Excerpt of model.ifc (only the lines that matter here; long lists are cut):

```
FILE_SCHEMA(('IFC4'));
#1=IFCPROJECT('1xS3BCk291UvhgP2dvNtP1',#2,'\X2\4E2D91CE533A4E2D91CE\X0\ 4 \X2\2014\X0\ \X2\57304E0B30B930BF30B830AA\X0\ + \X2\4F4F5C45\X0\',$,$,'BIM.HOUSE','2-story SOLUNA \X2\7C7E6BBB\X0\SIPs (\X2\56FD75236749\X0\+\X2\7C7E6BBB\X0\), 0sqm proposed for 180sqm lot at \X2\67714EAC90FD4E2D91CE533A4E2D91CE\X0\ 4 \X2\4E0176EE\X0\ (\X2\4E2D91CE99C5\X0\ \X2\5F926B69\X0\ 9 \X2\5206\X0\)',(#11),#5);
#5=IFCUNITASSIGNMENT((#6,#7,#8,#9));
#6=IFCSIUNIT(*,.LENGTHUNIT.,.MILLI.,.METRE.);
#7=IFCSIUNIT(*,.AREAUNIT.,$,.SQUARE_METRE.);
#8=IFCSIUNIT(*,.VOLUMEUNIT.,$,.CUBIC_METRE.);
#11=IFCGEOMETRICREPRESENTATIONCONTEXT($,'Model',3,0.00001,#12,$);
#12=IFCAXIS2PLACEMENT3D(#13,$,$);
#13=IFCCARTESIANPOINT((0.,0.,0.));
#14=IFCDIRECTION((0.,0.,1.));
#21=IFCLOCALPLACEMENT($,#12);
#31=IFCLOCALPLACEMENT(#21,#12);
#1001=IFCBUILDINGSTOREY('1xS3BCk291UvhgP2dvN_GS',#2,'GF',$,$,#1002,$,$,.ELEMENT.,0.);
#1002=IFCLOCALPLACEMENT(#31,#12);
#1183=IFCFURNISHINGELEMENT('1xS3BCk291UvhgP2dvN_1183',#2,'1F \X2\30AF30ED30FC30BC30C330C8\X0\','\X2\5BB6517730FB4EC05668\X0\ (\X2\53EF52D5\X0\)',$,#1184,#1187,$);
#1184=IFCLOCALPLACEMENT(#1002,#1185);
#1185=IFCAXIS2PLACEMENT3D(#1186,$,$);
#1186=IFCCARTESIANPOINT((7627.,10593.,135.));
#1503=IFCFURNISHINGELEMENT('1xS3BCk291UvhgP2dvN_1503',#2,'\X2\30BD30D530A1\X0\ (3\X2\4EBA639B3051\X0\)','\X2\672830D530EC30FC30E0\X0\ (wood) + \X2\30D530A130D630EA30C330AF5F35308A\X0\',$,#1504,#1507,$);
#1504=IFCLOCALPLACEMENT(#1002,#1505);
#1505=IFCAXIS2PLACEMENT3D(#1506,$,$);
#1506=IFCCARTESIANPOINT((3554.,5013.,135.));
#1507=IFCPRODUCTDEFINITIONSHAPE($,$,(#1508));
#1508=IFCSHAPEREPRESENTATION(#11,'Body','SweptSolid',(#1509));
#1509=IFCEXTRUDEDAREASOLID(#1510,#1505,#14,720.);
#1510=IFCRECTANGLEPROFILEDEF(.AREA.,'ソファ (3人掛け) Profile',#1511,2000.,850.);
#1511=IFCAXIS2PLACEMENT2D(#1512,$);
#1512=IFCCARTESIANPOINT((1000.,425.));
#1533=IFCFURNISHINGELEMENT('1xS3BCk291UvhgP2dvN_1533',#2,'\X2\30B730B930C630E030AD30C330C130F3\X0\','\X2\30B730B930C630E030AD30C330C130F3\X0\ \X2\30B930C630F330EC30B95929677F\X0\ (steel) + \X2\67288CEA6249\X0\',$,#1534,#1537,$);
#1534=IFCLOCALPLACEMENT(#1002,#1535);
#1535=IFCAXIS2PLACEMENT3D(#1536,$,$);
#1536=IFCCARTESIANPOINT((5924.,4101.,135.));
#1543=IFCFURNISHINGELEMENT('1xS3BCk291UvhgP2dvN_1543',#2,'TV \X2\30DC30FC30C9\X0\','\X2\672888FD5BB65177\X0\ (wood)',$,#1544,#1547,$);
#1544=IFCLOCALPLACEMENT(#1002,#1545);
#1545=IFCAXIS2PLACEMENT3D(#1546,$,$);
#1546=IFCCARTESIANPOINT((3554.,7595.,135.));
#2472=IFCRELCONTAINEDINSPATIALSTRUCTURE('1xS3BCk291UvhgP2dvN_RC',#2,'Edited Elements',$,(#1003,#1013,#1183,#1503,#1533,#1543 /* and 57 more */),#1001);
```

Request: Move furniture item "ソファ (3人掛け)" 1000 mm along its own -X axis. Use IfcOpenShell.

```python
import ifcopenshell
import ifcopenshell.api.geometry
import ifcopenshell.util.placement
import ifcopenshell.util.unit

model = ifcopenshell.open("model.ifc")
unit_scale = ifcopenshell.util.unit.calculate_unit_scale(model)

item = model.by_guid("1xS3BCk291UvhgP2dvN_1503")
matrix = ifcopenshell.util.placement.get_local_placement(item.ObjectPlacement)
matrix[:3, 3] -= matrix[:3, 0] * 1 / unit_scale
ifcopenshell.api.geometry.edit_object_placement(model, product=item, matrix=matrix, is_si=False)

print(ifcopenshell.util.placement.get_local_placement(item.ObjectPlacement).round(3) + 0.0)

model.write("model_updated.ifc")
```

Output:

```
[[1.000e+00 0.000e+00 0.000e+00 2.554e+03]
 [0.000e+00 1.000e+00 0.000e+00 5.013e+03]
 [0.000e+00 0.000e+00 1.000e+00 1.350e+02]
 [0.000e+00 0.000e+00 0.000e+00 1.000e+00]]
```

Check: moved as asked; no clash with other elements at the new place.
